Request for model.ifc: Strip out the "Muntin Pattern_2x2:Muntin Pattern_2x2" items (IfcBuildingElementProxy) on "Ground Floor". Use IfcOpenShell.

First a look at what the model holds.

```python
import ifcopenshell
import ifcopenshell.util.element

model = ifcopenshell.open("model.ifc")
print(model.schema)
storey = next(s for s in model.by_type("IfcBuildingStorey") if s.Name == "Ground Floor")
proxies = [e for e in ifcopenshell.util.element.get_decomposition(storey) if e.is_a("IfcBuildingElementProxy")]
seen = {}
for e in proxies:
    element_type = ifcopenshell.util.element.get_type(e)
    name = element_type.Name if element_type not in (None, e) else None
    seen[name] = seen.get(name, 0) + 1
for name, count in sorted(seen.items(), key=str):
    print(count, "x", name)
```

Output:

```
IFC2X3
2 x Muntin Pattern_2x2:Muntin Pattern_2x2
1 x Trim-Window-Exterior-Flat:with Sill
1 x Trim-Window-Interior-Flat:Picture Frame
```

```python
import ifcopenshell
import ifcopenshell.api.root
import ifcopenshell.util.element

model = ifcopenshell.open("model.ifc")

storey = next(s for s in model.by_type("IfcBuildingStorey") if s.Name == "Ground Floor")
proxies = [e for e in ifcopenshell.util.element.get_decomposition(storey) if e.is_a("IfcBuildingElementProxy")]
targets = [e for e in proxies if (t := ifcopenshell.util.element.get_type(e)) not in (None, e) and t.Name == "Muntin Pattern_2x2:Muntin Pattern_2x2"]

for e in targets:
    ifcopenshell.api.root.remove_product(model, product=e)
print(len(targets), "removed")

model.write("model_edited.ifc")
```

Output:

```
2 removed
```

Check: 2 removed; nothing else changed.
